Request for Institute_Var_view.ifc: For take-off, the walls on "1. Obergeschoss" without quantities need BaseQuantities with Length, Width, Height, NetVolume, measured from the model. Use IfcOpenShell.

First a look at what the model holds.

```python
import ifcopenshell
import ifcopenshell.util.element
import ifcopenshell.util.unit

model = ifcopenshell.open("Institute_Var_view.ifc")
print(model.schema)
for unit_type in ("LENGTHUNIT", "AREAUNIT", "VOLUMEUNIT"):
    print(unit_type, ifcopenshell.util.unit.calculate_unit_scale(model, unit_type))
storey = next(s for s in model.by_type("IfcBuildingStorey") if s.Name == "1. Obergeschoss")
walls = [e for e in ifcopenshell.util.element.get_decomposition(storey) if e.is_a("IfcWall")]
for e in sorted(walls, key=lambda e: e.id()):
    print(e.id(), e.is_a(), e.Name, list(ifcopenshell.util.element.get_psets(e, qtos_only=True)), sep=" | ")
```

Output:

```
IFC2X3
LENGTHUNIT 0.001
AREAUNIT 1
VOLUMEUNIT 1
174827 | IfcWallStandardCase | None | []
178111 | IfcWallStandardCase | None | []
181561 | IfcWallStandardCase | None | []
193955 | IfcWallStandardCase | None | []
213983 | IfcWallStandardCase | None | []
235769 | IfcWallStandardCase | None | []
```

```python
import ifcopenshell
import ifcopenshell.api.pset
import ifcopenshell.geom
import ifcopenshell.util.element
import ifcopenshell.util.shape
import ifcopenshell.util.unit

model = ifcopenshell.open("Institute_Var_view.ifc")
unit_scale = ifcopenshell.util.unit.calculate_unit_scale(model)
volume_scale = ifcopenshell.util.unit.calculate_unit_scale(model, "VOLUMEUNIT")
settings = ifcopenshell.geom.settings()

storey = next(s for s in model.by_type("IfcBuildingStorey") if s.Name == "1. Obergeschoss")
walls = [e for e in ifcopenshell.util.element.get_decomposition(storey) if e.is_a("IfcWall")]

for e in sorted(walls, key=lambda e: e.id()):
    if ifcopenshell.util.element.get_psets(e, qtos_only=True, should_inherit=False):
        continue
    # Geometry comes back in metres, in the element's own axes.
    shape = ifcopenshell.geom.create_shape(settings, e)
    values = {
        "Length": ifcopenshell.util.shape.get_x(shape.geometry) / unit_scale,
        "Width": ifcopenshell.util.shape.get_y(shape.geometry) / unit_scale,
        "Height": ifcopenshell.util.shape.get_z(shape.geometry) / unit_scale,
        "NetVolume": ifcopenshell.util.shape.get_volume(shape.geometry) / volume_scale,
    }
    qto = ifcopenshell.api.pset.add_qto(model, product=e, name="BaseQuantities")
    ifcopenshell.api.pset.edit_qto(model, qto=qto, properties=values)
    print(e.id(), {k: round(v, 3) for k, v in values.items()})

model.write("Institute_Var_view-out.ifc")
```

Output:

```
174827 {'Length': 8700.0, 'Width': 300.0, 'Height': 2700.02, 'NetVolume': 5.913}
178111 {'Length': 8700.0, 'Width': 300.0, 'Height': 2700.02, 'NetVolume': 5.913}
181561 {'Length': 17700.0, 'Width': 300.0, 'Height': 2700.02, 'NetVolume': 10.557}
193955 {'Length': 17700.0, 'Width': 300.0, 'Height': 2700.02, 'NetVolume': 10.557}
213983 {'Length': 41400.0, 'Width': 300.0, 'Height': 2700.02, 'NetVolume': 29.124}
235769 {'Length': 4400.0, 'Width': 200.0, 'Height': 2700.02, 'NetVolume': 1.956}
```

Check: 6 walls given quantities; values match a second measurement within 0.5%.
